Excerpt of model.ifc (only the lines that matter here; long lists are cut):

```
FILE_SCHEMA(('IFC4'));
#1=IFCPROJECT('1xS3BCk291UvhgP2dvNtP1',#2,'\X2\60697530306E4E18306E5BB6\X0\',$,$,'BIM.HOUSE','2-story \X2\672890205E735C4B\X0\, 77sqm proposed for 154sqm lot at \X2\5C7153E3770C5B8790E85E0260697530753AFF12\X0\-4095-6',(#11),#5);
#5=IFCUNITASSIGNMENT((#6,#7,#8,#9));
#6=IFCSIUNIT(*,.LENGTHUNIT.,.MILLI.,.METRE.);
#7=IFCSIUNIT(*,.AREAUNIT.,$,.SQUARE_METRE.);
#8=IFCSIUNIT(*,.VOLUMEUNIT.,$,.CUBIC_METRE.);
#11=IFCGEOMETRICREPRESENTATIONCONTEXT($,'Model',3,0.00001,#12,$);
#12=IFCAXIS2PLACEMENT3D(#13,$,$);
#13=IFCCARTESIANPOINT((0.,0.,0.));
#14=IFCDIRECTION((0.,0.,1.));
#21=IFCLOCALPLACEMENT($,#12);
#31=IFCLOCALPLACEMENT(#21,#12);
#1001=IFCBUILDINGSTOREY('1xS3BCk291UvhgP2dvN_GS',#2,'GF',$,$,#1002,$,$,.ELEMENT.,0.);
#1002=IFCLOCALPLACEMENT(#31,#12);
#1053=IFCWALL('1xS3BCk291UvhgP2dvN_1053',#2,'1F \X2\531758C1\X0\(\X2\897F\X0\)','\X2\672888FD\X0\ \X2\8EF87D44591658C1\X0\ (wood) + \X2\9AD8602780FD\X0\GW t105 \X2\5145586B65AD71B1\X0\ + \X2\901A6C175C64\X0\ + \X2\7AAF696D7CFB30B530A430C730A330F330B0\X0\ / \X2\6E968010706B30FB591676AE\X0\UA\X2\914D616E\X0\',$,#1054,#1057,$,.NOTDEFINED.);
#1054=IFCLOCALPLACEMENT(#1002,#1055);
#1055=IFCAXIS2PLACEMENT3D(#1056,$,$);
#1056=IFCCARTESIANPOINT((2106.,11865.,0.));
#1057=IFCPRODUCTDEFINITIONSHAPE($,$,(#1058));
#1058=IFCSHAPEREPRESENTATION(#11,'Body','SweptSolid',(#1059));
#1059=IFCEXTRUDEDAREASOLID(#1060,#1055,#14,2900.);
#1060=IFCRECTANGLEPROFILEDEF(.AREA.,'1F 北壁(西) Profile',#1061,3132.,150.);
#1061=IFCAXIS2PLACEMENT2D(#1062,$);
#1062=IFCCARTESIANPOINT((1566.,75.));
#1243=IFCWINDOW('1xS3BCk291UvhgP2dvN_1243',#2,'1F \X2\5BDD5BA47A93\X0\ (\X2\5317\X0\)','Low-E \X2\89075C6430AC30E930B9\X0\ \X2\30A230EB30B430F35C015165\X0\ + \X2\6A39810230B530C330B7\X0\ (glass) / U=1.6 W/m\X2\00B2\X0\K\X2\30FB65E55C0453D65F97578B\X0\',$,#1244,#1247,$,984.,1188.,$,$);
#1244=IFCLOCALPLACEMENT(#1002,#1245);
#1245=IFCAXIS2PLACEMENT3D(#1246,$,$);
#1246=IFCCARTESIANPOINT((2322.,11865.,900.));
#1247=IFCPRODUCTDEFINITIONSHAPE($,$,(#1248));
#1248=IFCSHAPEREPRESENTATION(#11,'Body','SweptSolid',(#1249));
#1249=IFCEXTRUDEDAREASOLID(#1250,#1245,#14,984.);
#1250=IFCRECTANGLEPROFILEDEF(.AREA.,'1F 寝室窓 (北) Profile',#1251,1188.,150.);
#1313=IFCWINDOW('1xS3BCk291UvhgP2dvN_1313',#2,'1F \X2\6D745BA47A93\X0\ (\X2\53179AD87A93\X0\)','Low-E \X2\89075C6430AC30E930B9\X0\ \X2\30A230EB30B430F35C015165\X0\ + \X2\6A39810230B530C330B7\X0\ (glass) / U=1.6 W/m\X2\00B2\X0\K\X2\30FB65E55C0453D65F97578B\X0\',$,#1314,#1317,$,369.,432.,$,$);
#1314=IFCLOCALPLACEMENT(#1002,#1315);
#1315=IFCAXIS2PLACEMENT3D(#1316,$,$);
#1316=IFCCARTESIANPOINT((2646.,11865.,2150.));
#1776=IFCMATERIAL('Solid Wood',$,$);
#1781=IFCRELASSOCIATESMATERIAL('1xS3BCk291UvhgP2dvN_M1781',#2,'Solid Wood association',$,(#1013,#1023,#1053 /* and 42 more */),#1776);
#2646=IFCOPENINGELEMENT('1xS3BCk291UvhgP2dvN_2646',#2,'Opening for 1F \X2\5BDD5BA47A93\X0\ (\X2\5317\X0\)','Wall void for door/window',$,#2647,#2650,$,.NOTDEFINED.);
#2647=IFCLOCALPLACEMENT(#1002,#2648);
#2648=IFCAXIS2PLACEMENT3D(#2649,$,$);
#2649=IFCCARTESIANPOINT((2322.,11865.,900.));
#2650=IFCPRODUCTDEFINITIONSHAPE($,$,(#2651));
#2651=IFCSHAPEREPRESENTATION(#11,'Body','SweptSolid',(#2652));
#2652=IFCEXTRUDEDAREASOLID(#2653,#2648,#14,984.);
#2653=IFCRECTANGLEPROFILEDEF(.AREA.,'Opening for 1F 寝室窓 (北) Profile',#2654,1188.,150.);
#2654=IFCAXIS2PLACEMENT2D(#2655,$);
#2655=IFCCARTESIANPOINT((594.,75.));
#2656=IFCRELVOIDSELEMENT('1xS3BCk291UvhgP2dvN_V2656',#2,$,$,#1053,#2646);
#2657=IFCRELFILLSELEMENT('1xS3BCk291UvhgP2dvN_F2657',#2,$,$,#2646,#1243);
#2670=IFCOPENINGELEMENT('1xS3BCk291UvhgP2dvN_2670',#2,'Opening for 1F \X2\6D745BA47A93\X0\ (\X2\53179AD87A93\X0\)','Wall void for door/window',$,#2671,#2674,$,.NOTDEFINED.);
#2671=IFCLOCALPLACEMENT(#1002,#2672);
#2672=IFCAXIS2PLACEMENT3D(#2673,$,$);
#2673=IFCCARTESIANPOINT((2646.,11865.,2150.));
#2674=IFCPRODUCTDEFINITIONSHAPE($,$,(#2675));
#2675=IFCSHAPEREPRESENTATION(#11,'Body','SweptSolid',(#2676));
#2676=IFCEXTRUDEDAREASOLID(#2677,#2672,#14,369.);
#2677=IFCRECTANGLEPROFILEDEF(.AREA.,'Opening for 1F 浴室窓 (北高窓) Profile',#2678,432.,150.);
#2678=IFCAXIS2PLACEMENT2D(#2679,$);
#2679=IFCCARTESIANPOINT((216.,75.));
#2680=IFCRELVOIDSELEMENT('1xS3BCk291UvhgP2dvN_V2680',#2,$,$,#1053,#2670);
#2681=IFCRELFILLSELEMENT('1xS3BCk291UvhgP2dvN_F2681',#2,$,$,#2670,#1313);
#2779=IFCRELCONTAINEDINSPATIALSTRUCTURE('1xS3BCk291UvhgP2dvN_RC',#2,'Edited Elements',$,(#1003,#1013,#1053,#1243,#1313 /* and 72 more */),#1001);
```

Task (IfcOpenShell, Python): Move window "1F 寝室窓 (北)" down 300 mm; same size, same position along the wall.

```python
import numpy as np
import ifcopenshell
import ifcopenshell.api.geometry
import ifcopenshell.util.placement
import ifcopenshell.util.unit

model = ifcopenshell.open("model.ifc")
unit_scale = ifcopenshell.util.unit.calculate_unit_scale(model)

window = model.by_guid("1xS3BCk291UvhgP2dvN_1243")
opening = window.FillsVoids[0].RelatingOpeningElement
dz = -300.0

shift = np.array([0.0, 0.0, dz])
# The window is not placed relative to its opening, so move both.
for product in (opening, window):
    matrix = ifcopenshell.util.placement.get_local_placement(product.ObjectPlacement)
    matrix[:3, 3] += shift
    ifcopenshell.api.geometry.edit_object_placement(model, product=product, matrix=matrix, is_si=False)

print(f"moved by {dz * unit_scale:+.3f} m")

model.write("model_edited.ifc")
```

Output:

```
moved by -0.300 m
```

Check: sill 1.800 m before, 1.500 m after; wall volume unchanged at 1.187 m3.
